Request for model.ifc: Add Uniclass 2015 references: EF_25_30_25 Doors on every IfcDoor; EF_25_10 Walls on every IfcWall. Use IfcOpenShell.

First a look at what the model holds.

```python
import ifcopenshell

model = ifcopenshell.open("model.ifc")
print(model.schema)
print("classifications:", [c.Name for c in model.by_type("IfcClassification")])
for ifc_class in ("IfcDoor", "IfcRoof", "IfcStair", "IfcWall", "IfcWindow"):
    print(ifc_class, len(model.by_type(ifc_class)))
```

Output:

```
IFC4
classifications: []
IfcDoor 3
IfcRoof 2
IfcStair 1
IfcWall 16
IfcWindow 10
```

```python
import ifcopenshell
import ifcopenshell.api.classification

model = ifcopenshell.open("model.ifc")

system = ifcopenshell.api.classification.add_classification(model, classification="Uniclass 2015")

codes = {
    "IfcDoor": ("EF_25_30_25", "Doors"),
    "IfcWall": ("EF_25_10", "Walls"),
}
for ifc_class, (code, name) in codes.items():
    products = model.by_type(ifc_class)
    ifcopenshell.api.classification.add_reference(
        model, products=products, classification=system, identification=code, name=name
    )
    print(code, len(products))

model.write("model_updated.ifc")
```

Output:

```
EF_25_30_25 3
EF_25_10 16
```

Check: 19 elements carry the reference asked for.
